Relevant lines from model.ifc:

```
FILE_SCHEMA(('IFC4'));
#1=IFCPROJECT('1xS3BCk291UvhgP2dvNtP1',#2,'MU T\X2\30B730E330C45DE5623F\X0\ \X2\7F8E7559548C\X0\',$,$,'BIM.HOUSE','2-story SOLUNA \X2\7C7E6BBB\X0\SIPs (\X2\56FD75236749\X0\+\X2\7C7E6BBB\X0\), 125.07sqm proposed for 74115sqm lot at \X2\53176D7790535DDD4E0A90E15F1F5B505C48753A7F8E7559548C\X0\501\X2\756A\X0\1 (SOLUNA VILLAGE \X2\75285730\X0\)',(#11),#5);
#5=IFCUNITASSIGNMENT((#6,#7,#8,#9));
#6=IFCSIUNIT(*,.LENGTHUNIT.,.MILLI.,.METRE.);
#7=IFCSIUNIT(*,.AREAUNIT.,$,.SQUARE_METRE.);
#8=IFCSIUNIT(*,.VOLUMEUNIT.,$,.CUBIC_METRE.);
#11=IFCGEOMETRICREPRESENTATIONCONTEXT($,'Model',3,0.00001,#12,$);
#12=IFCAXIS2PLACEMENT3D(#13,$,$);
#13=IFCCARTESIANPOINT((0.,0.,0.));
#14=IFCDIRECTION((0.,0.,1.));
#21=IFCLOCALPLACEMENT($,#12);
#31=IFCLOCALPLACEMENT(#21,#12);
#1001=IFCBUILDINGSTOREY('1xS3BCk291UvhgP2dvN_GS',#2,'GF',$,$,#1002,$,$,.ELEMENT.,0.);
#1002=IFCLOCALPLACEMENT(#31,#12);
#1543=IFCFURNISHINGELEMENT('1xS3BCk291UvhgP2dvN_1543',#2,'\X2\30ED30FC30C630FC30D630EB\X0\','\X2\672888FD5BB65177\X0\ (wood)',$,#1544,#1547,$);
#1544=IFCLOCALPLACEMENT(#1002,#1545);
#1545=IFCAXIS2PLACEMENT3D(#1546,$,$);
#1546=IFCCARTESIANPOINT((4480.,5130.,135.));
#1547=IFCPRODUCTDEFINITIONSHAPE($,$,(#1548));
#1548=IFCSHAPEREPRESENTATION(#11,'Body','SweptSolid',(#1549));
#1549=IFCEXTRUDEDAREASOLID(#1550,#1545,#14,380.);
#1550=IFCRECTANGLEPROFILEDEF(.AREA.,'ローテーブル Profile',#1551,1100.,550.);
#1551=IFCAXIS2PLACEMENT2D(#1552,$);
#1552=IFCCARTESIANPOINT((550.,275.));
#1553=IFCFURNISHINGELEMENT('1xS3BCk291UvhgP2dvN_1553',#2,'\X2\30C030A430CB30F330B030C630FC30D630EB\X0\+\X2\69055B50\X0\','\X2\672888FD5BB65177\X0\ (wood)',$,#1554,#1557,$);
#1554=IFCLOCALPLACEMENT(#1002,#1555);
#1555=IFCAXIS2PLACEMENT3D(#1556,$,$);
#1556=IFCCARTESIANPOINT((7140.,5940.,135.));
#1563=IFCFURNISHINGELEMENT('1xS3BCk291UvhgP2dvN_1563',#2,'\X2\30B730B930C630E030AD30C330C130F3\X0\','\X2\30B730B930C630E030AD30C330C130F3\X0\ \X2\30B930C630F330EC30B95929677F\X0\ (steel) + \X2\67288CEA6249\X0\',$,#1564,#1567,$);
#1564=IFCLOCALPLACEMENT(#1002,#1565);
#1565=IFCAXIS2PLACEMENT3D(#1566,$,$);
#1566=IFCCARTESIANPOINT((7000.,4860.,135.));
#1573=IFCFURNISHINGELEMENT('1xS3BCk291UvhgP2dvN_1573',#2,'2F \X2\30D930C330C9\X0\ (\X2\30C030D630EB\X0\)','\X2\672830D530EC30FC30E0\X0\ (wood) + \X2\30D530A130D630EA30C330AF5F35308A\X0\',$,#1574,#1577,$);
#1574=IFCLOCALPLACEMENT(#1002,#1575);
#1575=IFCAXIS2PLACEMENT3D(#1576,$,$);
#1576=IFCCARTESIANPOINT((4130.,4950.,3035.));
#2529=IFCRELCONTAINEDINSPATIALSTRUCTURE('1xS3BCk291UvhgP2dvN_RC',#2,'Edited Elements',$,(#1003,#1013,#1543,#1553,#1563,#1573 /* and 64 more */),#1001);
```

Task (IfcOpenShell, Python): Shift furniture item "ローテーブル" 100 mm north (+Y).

```python
import ifcopenshell
import ifcopenshell.api.geometry
import ifcopenshell.util.placement
import ifcopenshell.util.unit

model = ifcopenshell.open("model.ifc")
unit_scale = ifcopenshell.util.unit.calculate_unit_scale(model)

item = model.by_id(1543)
matrix = ifcopenshell.util.placement.get_local_placement(item.ObjectPlacement)
matrix[1, 3] += 0.1 / unit_scale
ifcopenshell.api.geometry.edit_object_placement(model, product=item, matrix=matrix, is_si=False)

print(ifcopenshell.util.placement.get_local_placement(item.ObjectPlacement).round(3) + 0.0)

model.write("model-out.ifc")
```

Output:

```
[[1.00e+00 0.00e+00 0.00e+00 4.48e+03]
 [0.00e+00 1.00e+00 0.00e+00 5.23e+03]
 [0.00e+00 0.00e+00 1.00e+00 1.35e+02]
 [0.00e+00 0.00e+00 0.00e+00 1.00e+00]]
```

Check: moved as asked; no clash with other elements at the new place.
